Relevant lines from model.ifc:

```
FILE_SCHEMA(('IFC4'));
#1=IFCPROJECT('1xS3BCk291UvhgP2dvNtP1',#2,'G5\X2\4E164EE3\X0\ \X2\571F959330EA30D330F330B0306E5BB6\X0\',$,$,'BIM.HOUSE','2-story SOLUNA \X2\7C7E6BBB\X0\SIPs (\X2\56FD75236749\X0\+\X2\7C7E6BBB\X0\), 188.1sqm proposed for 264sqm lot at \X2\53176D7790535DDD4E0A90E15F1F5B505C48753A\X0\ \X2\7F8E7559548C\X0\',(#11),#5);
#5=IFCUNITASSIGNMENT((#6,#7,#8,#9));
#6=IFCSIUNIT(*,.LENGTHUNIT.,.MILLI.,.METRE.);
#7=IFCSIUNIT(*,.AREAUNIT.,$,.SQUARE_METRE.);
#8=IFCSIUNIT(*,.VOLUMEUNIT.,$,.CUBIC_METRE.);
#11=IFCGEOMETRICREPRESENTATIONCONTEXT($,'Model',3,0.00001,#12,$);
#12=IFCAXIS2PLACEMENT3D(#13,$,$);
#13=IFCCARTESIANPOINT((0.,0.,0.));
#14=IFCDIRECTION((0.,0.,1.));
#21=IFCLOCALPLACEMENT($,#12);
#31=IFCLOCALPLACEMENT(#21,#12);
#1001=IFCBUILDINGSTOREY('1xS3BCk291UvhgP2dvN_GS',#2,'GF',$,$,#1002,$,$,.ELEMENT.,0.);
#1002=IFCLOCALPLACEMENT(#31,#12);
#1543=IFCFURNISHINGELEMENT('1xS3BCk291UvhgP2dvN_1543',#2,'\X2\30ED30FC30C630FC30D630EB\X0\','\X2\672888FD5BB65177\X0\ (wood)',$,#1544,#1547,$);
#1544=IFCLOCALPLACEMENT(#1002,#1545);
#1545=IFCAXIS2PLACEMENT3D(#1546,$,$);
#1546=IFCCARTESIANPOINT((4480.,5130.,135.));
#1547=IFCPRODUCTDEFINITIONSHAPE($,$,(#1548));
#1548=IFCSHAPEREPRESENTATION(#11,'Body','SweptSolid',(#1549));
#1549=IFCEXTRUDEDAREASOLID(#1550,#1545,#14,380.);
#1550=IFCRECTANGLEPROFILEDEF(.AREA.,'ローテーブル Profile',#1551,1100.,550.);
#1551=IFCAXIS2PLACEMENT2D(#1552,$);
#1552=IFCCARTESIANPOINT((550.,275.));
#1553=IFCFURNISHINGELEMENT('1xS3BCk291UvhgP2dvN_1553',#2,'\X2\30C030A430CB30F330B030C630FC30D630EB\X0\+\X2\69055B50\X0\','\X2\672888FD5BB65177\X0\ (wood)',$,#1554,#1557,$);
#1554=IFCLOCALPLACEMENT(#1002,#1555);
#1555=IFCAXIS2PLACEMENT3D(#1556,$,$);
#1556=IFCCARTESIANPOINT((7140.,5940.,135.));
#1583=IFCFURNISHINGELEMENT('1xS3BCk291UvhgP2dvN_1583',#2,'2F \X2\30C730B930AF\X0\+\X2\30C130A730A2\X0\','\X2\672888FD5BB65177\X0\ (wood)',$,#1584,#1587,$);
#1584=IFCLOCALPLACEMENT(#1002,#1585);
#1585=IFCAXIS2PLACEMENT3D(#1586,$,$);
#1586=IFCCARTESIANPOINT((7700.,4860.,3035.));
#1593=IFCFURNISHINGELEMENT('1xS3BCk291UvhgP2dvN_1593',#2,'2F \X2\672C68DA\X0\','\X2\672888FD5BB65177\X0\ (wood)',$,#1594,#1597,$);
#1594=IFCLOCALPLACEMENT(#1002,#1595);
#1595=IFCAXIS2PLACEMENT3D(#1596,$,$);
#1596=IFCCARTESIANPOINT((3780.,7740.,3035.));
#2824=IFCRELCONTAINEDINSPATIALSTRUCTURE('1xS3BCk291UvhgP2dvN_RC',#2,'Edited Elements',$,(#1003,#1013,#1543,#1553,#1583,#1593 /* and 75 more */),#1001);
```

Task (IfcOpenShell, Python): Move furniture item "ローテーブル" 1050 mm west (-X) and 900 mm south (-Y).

```python
import ifcopenshell
import ifcopenshell.api.geometry
import ifcopenshell.util.placement
import ifcopenshell.util.unit

model = ifcopenshell.open("model.ifc")
unit_scale = ifcopenshell.util.unit.calculate_unit_scale(model)

item = model.by_guid("1xS3BCk291UvhgP2dvN_1543")
matrix = ifcopenshell.util.placement.get_local_placement(item.ObjectPlacement)
matrix[0, 3] -= 1.05 / unit_scale
matrix[1, 3] -= 0.9 / unit_scale
ifcopenshell.api.geometry.edit_object_placement(model, product=item, matrix=matrix, is_si=False)

print(ifcopenshell.util.placement.get_local_placement(item.ObjectPlacement).round(3) + 0.0)

model.write("model_edited.ifc")
```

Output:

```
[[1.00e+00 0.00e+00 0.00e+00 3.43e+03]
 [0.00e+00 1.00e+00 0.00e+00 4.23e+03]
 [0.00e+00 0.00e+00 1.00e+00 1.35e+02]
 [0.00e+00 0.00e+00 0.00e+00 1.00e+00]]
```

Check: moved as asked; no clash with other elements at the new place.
